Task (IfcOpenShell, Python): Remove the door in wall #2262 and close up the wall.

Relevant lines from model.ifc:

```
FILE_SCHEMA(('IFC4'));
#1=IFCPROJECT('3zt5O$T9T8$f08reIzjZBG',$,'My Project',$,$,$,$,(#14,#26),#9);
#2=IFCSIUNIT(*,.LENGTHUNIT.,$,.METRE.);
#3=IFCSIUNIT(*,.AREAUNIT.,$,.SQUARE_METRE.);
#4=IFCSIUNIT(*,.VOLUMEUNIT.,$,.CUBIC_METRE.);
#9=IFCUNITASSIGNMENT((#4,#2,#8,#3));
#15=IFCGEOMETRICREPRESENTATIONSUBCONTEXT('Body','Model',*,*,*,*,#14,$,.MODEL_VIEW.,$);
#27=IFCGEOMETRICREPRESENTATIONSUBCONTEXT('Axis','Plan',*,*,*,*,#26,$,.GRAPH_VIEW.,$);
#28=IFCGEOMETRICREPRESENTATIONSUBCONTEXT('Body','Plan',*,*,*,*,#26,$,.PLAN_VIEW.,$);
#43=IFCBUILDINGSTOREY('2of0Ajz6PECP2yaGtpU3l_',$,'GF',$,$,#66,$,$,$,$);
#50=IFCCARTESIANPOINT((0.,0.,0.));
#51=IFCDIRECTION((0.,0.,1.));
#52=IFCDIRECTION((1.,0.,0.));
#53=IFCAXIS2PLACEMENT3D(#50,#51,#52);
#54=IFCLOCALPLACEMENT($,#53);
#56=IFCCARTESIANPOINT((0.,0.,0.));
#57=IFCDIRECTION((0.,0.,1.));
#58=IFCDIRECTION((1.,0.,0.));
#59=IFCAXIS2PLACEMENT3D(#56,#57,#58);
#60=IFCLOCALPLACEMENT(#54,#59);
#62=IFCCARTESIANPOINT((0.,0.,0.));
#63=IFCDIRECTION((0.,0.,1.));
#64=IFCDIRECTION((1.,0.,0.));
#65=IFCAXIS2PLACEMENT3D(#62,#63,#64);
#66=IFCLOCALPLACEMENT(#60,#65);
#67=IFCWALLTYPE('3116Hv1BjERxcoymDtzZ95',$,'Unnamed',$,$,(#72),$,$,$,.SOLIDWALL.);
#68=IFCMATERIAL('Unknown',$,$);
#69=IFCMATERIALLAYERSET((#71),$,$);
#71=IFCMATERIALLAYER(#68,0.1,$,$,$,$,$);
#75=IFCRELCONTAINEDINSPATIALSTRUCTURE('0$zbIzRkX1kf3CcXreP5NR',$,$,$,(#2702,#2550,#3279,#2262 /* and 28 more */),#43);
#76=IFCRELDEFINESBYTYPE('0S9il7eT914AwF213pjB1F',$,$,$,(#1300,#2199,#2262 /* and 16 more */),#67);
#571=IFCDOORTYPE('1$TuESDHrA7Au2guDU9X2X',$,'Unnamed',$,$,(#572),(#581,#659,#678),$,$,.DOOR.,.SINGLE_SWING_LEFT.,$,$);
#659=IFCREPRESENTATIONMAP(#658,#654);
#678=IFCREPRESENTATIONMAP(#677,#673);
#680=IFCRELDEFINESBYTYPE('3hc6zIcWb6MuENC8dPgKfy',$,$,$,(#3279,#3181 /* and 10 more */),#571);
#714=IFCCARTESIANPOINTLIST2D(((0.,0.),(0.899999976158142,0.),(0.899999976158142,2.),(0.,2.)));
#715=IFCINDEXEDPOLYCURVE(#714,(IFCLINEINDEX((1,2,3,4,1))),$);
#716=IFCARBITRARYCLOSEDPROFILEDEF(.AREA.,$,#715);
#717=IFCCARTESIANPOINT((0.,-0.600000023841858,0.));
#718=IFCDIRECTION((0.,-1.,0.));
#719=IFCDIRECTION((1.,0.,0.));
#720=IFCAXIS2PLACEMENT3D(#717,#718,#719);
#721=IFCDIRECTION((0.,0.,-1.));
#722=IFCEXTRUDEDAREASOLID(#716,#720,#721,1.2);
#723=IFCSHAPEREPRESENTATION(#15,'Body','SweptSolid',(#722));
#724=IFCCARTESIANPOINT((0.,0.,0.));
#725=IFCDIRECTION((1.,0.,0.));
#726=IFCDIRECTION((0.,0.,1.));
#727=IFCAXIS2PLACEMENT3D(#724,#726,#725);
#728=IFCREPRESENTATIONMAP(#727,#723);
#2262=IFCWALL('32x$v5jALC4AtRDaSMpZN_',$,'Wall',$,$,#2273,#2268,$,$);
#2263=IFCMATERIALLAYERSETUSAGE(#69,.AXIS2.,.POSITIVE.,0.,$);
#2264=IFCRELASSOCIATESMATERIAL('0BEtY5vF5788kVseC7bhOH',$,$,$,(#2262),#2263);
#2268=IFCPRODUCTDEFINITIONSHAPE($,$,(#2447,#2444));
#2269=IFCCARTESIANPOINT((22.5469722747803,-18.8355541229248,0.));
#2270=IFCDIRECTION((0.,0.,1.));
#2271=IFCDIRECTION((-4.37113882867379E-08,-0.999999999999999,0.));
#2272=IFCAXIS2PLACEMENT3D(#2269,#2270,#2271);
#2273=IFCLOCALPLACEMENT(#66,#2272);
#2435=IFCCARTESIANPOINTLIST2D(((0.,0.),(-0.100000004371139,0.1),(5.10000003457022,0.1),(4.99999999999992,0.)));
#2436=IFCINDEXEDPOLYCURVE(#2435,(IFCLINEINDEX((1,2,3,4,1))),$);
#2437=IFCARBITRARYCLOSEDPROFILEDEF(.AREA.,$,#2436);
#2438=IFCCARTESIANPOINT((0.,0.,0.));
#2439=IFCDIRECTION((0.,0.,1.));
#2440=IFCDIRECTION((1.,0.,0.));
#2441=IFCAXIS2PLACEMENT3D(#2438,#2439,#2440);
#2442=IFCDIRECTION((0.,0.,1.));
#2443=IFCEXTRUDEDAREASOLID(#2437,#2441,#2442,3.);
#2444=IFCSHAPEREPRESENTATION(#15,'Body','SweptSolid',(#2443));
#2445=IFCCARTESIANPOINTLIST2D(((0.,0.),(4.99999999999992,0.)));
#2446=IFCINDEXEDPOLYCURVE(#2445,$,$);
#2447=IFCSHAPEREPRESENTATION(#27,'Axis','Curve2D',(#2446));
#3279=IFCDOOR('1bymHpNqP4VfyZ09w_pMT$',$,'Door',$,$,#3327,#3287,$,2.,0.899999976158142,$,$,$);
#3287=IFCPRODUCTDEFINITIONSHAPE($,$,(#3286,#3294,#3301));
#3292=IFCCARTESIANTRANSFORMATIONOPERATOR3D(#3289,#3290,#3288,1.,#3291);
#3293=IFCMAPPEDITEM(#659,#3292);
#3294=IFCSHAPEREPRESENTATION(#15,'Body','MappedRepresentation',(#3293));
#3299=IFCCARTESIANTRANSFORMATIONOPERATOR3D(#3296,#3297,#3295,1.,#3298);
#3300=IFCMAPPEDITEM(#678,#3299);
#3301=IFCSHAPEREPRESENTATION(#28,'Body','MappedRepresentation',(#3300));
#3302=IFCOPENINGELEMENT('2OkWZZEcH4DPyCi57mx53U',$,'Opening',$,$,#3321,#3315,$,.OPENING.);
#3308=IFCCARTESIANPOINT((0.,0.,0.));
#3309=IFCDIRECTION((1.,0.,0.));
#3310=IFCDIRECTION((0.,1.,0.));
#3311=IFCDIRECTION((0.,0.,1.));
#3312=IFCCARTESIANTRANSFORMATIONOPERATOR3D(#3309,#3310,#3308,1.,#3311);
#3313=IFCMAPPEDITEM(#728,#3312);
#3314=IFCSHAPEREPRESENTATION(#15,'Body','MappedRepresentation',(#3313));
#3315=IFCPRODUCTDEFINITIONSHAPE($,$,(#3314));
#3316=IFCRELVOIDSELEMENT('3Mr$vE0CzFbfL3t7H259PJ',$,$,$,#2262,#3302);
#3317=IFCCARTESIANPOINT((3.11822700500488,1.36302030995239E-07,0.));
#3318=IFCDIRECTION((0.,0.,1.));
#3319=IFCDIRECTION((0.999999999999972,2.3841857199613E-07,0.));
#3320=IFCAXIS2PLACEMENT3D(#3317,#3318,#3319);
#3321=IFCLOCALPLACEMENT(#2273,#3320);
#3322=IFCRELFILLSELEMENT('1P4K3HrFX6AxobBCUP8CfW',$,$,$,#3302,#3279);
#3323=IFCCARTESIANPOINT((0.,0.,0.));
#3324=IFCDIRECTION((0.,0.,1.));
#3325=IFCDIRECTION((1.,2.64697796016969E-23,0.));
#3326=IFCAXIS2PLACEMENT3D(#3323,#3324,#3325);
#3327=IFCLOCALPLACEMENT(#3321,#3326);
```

```python
import ifcopenshell
import ifcopenshell.api.feature
import ifcopenshell.api.root
import ifcopenshell.geom
import ifcopenshell.util.shape

model = ifcopenshell.open("model.ifc")
settings = ifcopenshell.geom.settings()


def volume(element):
    """Net volume in cubic metres, openings subtracted."""
    shape = ifcopenshell.geom.create_shape(settings, element)
    return ifcopenshell.util.shape.get_volume(shape.geometry)


door = model.by_guid("1bymHpNqP4VfyZ09w_pMT$")
opening = door.FillsVoids[0].RelatingOpeningElement
wall = opening.VoidsElements[0].RelatingBuildingElement
before = volume(wall)

ifcopenshell.api.root.remove_product(model, product=door)
ifcopenshell.api.feature.remove_feature(model, feature=opening)

after = volume(wall)

print(f"wall volume {before:.3f} -> {after:.3f} m3")

model.write("model_v2.ifc")
```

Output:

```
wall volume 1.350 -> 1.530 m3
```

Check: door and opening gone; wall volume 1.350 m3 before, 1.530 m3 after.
